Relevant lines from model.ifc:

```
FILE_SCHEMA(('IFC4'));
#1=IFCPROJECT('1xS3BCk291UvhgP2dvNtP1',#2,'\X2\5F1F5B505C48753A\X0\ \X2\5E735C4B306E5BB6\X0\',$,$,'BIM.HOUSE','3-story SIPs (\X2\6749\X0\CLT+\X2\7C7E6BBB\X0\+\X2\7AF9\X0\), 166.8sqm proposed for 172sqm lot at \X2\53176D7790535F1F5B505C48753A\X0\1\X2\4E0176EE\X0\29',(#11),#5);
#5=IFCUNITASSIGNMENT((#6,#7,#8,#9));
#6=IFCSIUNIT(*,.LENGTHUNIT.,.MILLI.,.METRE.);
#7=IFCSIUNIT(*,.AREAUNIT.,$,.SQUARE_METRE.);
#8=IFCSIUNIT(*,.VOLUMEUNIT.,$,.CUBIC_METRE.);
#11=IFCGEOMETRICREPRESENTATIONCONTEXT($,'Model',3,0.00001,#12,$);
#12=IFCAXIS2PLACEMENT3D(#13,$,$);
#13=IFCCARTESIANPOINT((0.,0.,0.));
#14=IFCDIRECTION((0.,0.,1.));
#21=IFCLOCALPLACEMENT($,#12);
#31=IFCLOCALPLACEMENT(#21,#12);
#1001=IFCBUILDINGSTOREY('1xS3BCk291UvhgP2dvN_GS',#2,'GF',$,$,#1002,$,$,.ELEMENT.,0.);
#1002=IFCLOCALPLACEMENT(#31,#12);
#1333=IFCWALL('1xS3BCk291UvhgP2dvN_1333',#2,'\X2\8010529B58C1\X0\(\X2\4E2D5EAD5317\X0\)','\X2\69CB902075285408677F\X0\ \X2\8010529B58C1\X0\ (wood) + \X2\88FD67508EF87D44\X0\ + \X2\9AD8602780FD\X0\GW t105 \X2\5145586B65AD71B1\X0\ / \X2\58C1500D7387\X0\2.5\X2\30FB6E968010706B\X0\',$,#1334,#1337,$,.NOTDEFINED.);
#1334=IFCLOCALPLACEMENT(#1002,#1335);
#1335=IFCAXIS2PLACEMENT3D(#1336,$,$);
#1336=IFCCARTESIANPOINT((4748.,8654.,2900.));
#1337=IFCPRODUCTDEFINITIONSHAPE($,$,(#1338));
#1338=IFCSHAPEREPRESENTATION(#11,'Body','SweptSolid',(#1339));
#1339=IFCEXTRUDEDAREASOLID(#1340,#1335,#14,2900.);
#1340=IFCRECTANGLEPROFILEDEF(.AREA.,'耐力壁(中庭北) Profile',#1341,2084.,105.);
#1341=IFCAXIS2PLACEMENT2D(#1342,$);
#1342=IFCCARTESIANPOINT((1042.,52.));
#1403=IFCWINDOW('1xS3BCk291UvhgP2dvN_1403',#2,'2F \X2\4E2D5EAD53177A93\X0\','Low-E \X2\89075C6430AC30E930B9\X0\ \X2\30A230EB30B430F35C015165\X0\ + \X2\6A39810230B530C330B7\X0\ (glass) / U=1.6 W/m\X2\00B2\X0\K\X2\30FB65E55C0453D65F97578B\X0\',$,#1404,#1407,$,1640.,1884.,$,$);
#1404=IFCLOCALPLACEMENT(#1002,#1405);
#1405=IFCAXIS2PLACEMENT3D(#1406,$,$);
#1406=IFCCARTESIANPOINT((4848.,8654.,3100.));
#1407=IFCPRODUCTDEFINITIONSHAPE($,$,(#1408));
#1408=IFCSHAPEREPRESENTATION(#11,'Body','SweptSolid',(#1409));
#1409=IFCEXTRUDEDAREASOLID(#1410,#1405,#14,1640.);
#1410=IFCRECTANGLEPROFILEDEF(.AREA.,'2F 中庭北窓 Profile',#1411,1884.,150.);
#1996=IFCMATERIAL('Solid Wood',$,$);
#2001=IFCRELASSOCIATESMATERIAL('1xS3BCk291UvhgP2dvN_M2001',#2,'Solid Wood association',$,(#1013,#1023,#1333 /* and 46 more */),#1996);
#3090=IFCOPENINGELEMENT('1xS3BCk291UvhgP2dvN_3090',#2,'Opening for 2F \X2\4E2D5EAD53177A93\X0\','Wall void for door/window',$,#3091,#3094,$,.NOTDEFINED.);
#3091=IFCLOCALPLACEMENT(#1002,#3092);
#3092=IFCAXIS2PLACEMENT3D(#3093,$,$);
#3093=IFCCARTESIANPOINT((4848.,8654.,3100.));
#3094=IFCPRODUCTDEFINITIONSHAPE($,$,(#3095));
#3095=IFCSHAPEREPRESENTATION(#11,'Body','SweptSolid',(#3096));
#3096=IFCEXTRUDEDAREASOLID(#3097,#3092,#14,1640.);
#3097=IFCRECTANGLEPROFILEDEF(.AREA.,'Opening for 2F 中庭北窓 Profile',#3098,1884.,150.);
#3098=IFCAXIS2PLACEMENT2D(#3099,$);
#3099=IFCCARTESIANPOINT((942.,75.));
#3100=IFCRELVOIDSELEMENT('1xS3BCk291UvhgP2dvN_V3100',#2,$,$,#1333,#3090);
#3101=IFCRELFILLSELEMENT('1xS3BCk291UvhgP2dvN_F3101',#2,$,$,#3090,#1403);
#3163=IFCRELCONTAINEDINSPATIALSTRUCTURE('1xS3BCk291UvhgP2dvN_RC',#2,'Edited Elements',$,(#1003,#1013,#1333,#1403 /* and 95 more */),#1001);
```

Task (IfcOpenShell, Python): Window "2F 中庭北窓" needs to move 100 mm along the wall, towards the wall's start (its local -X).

```python
import ifcopenshell
import ifcopenshell.api.geometry
import ifcopenshell.util.placement
import ifcopenshell.util.unit

model = ifcopenshell.open("model.ifc")
unit_scale = ifcopenshell.util.unit.calculate_unit_scale(model)

window = model.by_id(1403)
opening = window.FillsVoids[0].RelatingOpeningElement
wall = opening.VoidsElements[0].RelatingBuildingElement

wall_matrix = ifcopenshell.util.placement.get_local_placement(wall.ObjectPlacement)
shift = wall_matrix[:3, 0] * -0.1 / unit_scale
before = ifcopenshell.util.placement.get_local_placement(window.ObjectPlacement)[:3, 3].copy()

# The window is not placed relative to its opening, so move both.
for product in (opening, window):
    matrix = ifcopenshell.util.placement.get_local_placement(product.ObjectPlacement)
    matrix[:3, 3] += shift
    ifcopenshell.api.geometry.edit_object_placement(model, product=product, matrix=matrix, is_si=False)

after = ifcopenshell.util.placement.get_local_placement(window.ObjectPlacement)[:3, 3]
print("window moved by", (after - before).round(3) + 0.0)

model.write("model_v2.ifc")
```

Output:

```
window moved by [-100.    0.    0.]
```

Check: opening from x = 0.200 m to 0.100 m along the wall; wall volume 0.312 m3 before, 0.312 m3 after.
